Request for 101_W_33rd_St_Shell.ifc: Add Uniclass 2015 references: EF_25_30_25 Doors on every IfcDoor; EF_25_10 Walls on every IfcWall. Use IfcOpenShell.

First a look at what the model holds.

```python
import ifcopenshell

model = ifcopenshell.open("101_W_33rd_St_Shell.ifc")
print(model.schema)
print("classifications:", [c.Name for c in model.by_type("IfcClassification")])
for ifc_class in ("IfcDoor", "IfcRoof", "IfcStair", "IfcWall", "IfcWindow"):
    print(ifc_class, len(model.by_type(ifc_class)))
```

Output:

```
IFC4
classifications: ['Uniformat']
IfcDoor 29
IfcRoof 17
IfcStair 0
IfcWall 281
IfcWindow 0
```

```python
import ifcopenshell
import ifcopenshell.api.classification

model = ifcopenshell.open("101_W_33rd_St_Shell.ifc")

system = ifcopenshell.api.classification.add_classification(model, classification="Uniclass 2015")

codes = {
    "IfcDoor": ("EF_25_30_25", "Doors"),
    "IfcWall": ("EF_25_10", "Walls"),
}
for ifc_class, (code, name) in codes.items():
    products = model.by_type(ifc_class)
    ifcopenshell.api.classification.add_reference(
        model, products=products, classification=system, identification=code, name=name
    )
    print(code, len(products))

model.write("101_W_33rd_St_Shell_rev.ifc")
```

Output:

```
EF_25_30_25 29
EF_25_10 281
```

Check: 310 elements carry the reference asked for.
